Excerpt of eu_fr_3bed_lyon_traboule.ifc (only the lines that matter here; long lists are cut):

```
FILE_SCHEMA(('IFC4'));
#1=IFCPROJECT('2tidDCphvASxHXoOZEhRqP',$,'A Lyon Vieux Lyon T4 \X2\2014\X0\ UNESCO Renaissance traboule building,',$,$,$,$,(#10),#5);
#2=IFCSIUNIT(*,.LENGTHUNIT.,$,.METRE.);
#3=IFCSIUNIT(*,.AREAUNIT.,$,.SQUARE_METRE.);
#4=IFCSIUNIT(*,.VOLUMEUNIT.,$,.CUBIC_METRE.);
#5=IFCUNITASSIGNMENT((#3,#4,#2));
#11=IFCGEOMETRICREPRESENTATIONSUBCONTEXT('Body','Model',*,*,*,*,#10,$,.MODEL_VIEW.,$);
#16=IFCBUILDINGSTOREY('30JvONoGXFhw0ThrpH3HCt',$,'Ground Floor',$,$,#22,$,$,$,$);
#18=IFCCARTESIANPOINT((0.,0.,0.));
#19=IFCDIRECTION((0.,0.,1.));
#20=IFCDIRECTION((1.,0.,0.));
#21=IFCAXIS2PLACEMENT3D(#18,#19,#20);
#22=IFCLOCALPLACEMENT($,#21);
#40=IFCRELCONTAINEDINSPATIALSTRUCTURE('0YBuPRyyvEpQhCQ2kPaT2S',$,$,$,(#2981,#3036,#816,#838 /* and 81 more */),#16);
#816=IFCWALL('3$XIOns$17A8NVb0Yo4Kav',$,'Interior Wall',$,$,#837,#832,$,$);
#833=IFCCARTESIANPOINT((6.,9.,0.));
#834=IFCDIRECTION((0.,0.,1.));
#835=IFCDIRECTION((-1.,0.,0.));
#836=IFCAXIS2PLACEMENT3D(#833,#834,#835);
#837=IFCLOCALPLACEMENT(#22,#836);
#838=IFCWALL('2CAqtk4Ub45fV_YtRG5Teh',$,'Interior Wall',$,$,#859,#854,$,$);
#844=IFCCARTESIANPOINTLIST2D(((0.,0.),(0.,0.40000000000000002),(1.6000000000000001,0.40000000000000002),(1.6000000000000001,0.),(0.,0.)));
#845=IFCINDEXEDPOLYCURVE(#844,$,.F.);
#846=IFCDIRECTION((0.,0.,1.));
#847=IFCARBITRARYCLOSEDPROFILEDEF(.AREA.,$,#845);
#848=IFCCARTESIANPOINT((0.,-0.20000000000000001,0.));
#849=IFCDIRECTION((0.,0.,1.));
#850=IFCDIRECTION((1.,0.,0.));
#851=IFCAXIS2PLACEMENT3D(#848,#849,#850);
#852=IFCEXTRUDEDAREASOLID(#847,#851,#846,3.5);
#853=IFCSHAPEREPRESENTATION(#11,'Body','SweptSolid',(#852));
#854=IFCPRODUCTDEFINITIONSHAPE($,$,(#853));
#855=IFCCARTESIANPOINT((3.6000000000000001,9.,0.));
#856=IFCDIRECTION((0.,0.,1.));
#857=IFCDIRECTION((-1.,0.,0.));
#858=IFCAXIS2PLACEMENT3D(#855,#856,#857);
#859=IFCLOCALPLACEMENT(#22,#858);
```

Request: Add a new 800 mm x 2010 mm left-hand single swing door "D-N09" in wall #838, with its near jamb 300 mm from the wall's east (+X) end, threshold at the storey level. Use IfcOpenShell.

```python
import numpy as np
import ifcopenshell
import ifcopenshell.api.feature
import ifcopenshell.api.geometry
import ifcopenshell.api.root
import ifcopenshell.api.spatial
import ifcopenshell.geom
import ifcopenshell.util.element
import ifcopenshell.util.placement
import ifcopenshell.util.representation
import ifcopenshell.util.shape
import ifcopenshell.util.unit

model = ifcopenshell.open("eu_fr_3bed_lyon_traboule.ifc")
unit_scale = ifcopenshell.util.unit.calculate_unit_scale(model)
settings = ifcopenshell.geom.settings()


def volume(element):
    """Net volume in cubic metres, openings subtracted."""
    shape = ifcopenshell.geom.create_shape(settings, element)
    return ifcopenshell.util.shape.get_volume(shape.geometry)


wall = model.by_guid("2CAqtk4Ub45fV_YtRG5Teh")
storey = ifcopenshell.util.element.get_container(wall, ifc_class="IfcBuildingStorey")
context = ifcopenshell.util.representation.get_context(model, "Model", "Body", "MODEL_VIEW")
before = volume(wall)

width, height, from_end, sill = 0.8, 2.01, 0.3, 0.0  # metres

# The wall runs along its own X axis, and the end named is its -X end.
wall_shape = ifcopenshell.geom.create_shape(settings, wall)
x, y, z = ifcopenshell.util.shape.get_vertices(wall_shape.geometry).T
start = x.min() + from_end
face, thickness = float(y.min()), float(y.max() - y.min())
wall_matrix = ifcopenshell.util.placement.get_local_placement(wall.ObjectPlacement)
level = ifcopenshell.util.placement.get_local_placement(storey.ObjectPlacement)[2, 3]


def in_wall(x, y):
    """Placement at x, y metres in the wall's axes, at sill height."""
    matrix = wall_matrix.copy()
    matrix[:, 3] = wall_matrix @ np.array([x / unit_scale, y / unit_scale, 0.0, 1.0])
    matrix[2, 3] = level + sill / unit_scale
    return matrix


# Opening: a box that overshoots both wall faces by 50 mm.
opening = ifcopenshell.api.root.create_entity(model, ifc_class="IfcOpeningElement", predefined_type="OPENING")
box = ifcopenshell.api.geometry.add_wall_representation(
    model, context=context, length=width, height=height, thickness=thickness + 0.1
)
ifcopenshell.api.geometry.assign_representation(model, product=opening, representation=box)
ifcopenshell.api.geometry.edit_object_placement(model, product=opening, matrix=in_wall(start, face - 0.05), is_si=False)
ifcopenshell.api.feature.add_feature(model, feature=opening, element=wall)

door = ifcopenshell.api.root.create_entity(model, ifc_class="IfcDoor", name="D-N09", predefined_type="DOOR")
door.OverallWidth, door.OverallHeight = width / unit_scale, height / unit_scale
door.OperationType = "SINGLE_SWING_LEFT"
body = ifcopenshell.api.geometry.add_door_representation(
    model,
    context=context,
    overall_width=door.OverallWidth,
    overall_height=door.OverallHeight,
    operation_type="SINGLE_SWING_LEFT",
    lining_properties={"LiningDepth": thickness / unit_scale, "ThresholdDepth": thickness / unit_scale},
)
ifcopenshell.api.geometry.assign_representation(model, product=door, representation=body)
ifcopenshell.api.spatial.assign_container(model, products=[door], relating_structure=storey)
ifcopenshell.api.feature.add_filling(model, opening=opening, element=door)

# The lining spans the wall, so the door starts at the wall face.
ifcopenshell.api.geometry.edit_object_placement(model, product=door, matrix=in_wall(start, face), is_si=False)

after = volume(wall)

print(f"wall volume {before:.3f} -> {after:.3f} m3")

model.write("eu_fr_3bed_lyon_traboule-out.ifc")
```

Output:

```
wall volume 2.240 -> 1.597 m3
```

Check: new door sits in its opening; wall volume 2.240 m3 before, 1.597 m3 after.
